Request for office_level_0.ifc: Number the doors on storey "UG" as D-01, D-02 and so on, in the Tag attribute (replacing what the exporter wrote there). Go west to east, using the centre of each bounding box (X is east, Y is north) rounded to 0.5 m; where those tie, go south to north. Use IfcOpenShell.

First a look at what the model holds.

```python
import ifcopenshell
import ifcopenshell.util.element
import ifcopenshell.util.placement

model = ifcopenshell.open("office_level_0.ifc")
print(model.schema)
storey = next(s for s in model.by_type("IfcBuildingStorey") if s.Name == "UG")
doors = [e for e in ifcopenshell.util.element.get_decomposition(storey) if e.is_a("IfcDoor")]
for e in sorted(doors, key=lambda e: e.id()):
    origin = ifcopenshell.util.placement.get_local_placement(e.ObjectPlacement)[:3, 3]
    print(e.id(), e.Tag, e.Name, origin.round(2) + 0.0, sep=" | ")
```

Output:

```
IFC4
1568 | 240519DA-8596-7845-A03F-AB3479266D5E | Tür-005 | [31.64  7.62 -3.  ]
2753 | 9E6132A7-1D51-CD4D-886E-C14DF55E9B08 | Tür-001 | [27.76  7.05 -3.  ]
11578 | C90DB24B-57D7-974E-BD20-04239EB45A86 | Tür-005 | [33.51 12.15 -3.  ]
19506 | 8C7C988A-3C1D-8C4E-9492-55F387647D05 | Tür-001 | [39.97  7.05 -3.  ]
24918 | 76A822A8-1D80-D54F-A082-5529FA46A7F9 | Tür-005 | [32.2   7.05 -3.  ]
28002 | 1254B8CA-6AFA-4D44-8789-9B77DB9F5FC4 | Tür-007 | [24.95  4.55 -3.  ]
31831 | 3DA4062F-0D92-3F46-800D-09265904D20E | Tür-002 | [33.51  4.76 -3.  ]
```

```python
import ifcopenshell
import ifcopenshell.geom
import ifcopenshell.util.element
import ifcopenshell.util.shape

model = ifcopenshell.open("office_level_0.ifc")
settings = ifcopenshell.geom.settings()
settings.set("use-world-coords", True)


def centre(element):
    shape = ifcopenshell.geom.create_shape(settings, element)
    return ifcopenshell.util.shape.get_bbox_centroid(shape.geometry)


storey = next(s for s in model.by_type("IfcBuildingStorey") if s.Name == "UG")
doors = [e for e in ifcopenshell.util.element.get_decomposition(storey) if e.is_a("IfcDoor")]

# Insertion points can sit at a corner or the storey origin, so sort by the geometry (in metres).
centres = {e: centre(e) for e in doors}
doors.sort(key=lambda e: (round(centres[e][0] / 0.5), centres[e][1]))

for i, e in enumerate(doors, start=1):
    number = f"D-{i:02d}"
    e.Tag = number
    print(e.id(), number)

model.write("office_level_0-out.ifc")
```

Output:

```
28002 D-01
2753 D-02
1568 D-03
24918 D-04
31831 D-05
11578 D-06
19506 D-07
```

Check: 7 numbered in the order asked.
